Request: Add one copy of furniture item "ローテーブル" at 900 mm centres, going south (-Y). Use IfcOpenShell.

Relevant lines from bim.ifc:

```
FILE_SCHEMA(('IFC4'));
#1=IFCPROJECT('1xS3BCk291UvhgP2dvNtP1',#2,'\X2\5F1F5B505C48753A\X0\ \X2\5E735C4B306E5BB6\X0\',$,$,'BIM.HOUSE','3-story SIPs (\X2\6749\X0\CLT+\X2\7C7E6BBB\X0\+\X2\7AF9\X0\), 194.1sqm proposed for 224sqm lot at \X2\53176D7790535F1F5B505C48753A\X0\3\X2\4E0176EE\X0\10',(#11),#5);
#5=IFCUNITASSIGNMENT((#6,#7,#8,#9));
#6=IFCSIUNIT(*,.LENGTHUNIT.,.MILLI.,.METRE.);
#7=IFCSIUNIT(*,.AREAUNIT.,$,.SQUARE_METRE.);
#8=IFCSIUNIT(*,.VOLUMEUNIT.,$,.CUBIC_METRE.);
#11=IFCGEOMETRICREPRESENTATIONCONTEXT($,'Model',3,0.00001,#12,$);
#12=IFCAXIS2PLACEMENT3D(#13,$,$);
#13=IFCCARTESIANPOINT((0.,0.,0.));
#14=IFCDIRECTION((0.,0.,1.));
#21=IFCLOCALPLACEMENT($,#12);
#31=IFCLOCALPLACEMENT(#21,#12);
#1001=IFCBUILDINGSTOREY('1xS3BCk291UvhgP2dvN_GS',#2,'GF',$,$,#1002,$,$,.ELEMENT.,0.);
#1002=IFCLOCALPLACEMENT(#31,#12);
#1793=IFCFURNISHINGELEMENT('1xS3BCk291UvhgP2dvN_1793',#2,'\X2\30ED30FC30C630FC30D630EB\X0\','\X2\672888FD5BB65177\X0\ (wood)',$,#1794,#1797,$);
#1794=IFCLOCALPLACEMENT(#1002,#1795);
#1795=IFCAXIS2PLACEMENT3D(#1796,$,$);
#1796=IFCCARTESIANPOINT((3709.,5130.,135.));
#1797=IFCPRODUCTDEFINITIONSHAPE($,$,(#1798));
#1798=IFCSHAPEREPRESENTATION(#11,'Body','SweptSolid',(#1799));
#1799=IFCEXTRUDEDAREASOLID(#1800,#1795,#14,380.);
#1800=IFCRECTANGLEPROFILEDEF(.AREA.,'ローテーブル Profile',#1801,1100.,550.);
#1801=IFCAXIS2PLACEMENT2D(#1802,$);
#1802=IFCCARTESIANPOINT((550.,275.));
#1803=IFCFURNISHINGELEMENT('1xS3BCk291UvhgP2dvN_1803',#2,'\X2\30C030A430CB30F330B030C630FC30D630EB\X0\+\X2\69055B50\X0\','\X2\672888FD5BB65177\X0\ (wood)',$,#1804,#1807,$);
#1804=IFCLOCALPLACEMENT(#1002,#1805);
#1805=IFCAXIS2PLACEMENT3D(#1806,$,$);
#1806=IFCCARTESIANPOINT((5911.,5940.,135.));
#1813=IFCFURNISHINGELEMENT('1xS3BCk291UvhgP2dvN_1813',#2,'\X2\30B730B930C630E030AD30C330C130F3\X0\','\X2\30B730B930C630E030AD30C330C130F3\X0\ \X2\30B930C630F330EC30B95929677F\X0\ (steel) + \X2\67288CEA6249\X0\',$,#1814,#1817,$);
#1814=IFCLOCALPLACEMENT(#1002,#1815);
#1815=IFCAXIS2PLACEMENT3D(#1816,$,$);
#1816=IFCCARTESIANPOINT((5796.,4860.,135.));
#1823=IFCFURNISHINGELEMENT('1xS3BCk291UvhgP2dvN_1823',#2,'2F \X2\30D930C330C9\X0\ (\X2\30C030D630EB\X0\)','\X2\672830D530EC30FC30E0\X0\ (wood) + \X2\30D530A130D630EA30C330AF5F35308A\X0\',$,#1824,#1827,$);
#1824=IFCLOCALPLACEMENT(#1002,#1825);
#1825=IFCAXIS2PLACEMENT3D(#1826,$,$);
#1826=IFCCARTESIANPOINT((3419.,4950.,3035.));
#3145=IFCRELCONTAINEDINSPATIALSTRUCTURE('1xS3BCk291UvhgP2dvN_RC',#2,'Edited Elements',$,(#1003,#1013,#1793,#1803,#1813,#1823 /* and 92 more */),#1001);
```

```python
import numpy as np
import ifcopenshell
import ifcopenshell.api.geometry
import ifcopenshell.api.root
import ifcopenshell.util.element
import ifcopenshell.util.placement

model = ifcopenshell.open("bim.ifc")


def reuse_history(source, copy):
    """copy_class also copies each property set's owner history, people and application; keep the originals."""
    for rel in copy.IsDefinedBy:
        if rel.is_a("IfcRelDefinesByProperties") and (history := rel.RelatingPropertyDefinition.OwnerHistory):
            rel.RelatingPropertyDefinition.OwnerHistory = source.OwnerHistory
            ifcopenshell.util.element.remove_deep2(model, history)


source = model.by_guid("1xS3BCk291UvhgP2dvN_1793")
base = ifcopenshell.util.placement.get_local_placement(source.ObjectPlacement)
step = np.array([0.0, -1.0, 0.0]) * 900.0

for i in range(1, 2):
    copy = ifcopenshell.api.root.copy_class(model, product=source)
    copy.Representation = ifcopenshell.util.element.copy_deep(
        model, source.Representation, exclude=["IfcGeometricRepresentationContext", "IfcRepresentationMap"]
    )
    reuse_history(source, copy)
    matrix = base.copy()
    matrix[:3, 3] += i * step
    print("added at", matrix[:3, 3].round(3) + 0.0)
    ifcopenshell.api.geometry.edit_object_placement(model, product=copy, matrix=matrix, is_si=False)

model.write("bim_v2.ifc")
```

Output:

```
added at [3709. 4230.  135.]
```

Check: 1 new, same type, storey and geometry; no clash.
